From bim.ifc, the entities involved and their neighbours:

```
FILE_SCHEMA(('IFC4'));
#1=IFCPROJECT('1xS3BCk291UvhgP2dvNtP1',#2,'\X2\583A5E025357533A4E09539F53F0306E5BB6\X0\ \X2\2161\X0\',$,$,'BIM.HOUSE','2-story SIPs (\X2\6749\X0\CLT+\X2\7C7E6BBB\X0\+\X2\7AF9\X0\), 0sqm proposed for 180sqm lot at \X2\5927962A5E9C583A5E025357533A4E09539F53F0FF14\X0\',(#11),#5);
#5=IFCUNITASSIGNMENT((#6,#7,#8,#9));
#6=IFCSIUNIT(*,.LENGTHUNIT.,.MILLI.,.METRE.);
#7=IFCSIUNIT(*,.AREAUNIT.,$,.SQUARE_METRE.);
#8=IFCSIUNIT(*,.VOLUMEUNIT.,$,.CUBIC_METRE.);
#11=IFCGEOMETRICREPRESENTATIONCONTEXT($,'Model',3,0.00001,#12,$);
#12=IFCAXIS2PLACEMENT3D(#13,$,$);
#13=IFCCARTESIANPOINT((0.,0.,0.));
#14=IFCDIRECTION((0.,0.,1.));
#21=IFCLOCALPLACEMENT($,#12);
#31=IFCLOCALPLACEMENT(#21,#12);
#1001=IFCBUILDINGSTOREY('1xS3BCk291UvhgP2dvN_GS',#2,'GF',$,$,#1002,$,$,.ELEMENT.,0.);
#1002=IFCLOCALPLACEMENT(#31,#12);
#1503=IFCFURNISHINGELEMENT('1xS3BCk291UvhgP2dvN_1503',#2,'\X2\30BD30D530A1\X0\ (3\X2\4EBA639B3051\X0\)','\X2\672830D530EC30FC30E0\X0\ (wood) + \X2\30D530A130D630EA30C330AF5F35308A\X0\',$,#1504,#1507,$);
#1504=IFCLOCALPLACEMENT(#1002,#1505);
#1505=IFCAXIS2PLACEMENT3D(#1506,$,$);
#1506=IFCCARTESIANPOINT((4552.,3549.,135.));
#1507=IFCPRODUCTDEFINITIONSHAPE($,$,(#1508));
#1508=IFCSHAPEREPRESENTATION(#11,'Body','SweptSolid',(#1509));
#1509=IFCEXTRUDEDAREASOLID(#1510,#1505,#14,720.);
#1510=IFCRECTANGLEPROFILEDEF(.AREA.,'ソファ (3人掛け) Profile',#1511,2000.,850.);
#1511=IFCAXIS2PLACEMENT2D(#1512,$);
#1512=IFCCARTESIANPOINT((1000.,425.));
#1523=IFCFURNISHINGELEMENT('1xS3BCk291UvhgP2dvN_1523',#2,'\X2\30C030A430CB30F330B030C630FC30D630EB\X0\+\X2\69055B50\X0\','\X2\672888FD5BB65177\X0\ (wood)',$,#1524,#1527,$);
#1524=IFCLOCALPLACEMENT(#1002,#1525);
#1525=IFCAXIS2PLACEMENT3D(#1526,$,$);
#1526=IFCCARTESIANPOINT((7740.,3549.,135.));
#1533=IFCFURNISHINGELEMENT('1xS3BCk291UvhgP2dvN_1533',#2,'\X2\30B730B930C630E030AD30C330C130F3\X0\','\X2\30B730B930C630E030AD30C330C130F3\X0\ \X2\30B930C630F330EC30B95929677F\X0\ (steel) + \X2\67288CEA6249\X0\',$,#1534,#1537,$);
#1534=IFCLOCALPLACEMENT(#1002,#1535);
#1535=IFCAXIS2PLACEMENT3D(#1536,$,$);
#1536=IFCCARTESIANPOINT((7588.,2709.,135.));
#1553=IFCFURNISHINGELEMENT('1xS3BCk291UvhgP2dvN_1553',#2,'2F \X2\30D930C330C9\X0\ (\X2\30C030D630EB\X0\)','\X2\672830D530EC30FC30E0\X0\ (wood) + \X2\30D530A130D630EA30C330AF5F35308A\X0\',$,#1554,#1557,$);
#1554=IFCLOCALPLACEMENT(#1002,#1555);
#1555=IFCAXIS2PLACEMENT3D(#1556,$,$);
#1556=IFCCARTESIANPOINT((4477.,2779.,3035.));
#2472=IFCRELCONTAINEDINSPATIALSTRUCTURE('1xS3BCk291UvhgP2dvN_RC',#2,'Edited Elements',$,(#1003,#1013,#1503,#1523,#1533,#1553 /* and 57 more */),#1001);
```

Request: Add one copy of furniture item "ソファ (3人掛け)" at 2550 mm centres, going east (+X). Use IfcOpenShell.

```python
import numpy as np
import ifcopenshell
import ifcopenshell.api.geometry
import ifcopenshell.api.root
import ifcopenshell.util.element
import ifcopenshell.util.placement

model = ifcopenshell.open("bim.ifc")


def reuse_history(source, copy):
    """copy_class also copies each property set's owner history, people and application; keep the originals."""
    for rel in copy.IsDefinedBy:
        if rel.is_a("IfcRelDefinesByProperties") and (history := rel.RelatingPropertyDefinition.OwnerHistory):
            rel.RelatingPropertyDefinition.OwnerHistory = source.OwnerHistory
            ifcopenshell.util.element.remove_deep2(model, history)


source = model.by_id(1503)
base = ifcopenshell.util.placement.get_local_placement(source.ObjectPlacement)
step = np.array([1.0, 0.0, 0.0]) * 2550.0

for i in range(1, 2):
    copy = ifcopenshell.api.root.copy_class(model, product=source)
    copy.Representation = ifcopenshell.util.element.copy_deep(
        model, source.Representation, exclude=["IfcGeometricRepresentationContext", "IfcRepresentationMap"]
    )
    reuse_history(source, copy)
    matrix = base.copy()
    matrix[:3, 3] += i * step
    print("added at", matrix[:3, 3].round(3) + 0.0)
    ifcopenshell.api.geometry.edit_object_placement(model, product=copy, matrix=matrix, is_si=False)

model.write("bim_edited.ifc")
```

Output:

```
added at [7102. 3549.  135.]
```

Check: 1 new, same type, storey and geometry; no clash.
